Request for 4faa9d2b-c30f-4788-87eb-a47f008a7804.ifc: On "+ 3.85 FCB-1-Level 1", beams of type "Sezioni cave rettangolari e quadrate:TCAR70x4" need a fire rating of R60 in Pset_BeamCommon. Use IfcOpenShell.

First a look at what the model holds.

```python
import ifcopenshell
import ifcopenshell.util.element

model = ifcopenshell.open("4faa9d2b-c30f-4788-87eb-a47f008a7804.ifc")
print(model.schema)
storey = next(s for s in model.by_type("IfcBuildingStorey") if s.Name == "+ 3.85 FCB-1-Level 1")
beams = [e for e in ifcopenshell.util.element.get_decomposition(storey) if e.is_a("IfcBeam")]
seen = {}
for e in beams:
    element_type = ifcopenshell.util.element.get_type(e)
    key = (element_type.Name if element_type != e and element_type else None, ifcopenshell.util.element.get_pset(e, "Pset_BeamCommon", "FireRating"))
    seen[key] = seen.get(key, 0) + 1
for (name, value), count in sorted(seen.items(), key=str):
    print(count, "x", name, "|", value)
```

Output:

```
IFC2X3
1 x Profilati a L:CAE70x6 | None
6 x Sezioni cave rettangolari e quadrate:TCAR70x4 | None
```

```python
import ifcopenshell
import ifcopenshell.api.pset
import ifcopenshell.util.element

model = ifcopenshell.open("4faa9d2b-c30f-4788-87eb-a47f008a7804.ifc")

storey = next(s for s in model.by_type("IfcBuildingStorey") if s.Name == "+ 3.85 FCB-1-Level 1")
beams = [e for e in ifcopenshell.util.element.get_decomposition(storey) if e.is_a("IfcBeam")]

count = 0
for e in beams:
    element_type = ifcopenshell.util.element.get_type(e)
    if element_type in (None, e) or element_type.Name != "Sezioni cave rettangolari e quadrate:TCAR70x4":
        continue
    # add_pset returns the element's existing set when there is one.
    pset = ifcopenshell.api.pset.add_pset(model, product=e, name="Pset_BeamCommon")
    ifcopenshell.api.pset.edit_pset(model, pset=pset, properties={"FireRating": "R60"})
    count += 1

print(count, "beams updated")

model.write("4faa9d2b-c30f-4788-87eb-a47f008a7804_updated.ifc")
```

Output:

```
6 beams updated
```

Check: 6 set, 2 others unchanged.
